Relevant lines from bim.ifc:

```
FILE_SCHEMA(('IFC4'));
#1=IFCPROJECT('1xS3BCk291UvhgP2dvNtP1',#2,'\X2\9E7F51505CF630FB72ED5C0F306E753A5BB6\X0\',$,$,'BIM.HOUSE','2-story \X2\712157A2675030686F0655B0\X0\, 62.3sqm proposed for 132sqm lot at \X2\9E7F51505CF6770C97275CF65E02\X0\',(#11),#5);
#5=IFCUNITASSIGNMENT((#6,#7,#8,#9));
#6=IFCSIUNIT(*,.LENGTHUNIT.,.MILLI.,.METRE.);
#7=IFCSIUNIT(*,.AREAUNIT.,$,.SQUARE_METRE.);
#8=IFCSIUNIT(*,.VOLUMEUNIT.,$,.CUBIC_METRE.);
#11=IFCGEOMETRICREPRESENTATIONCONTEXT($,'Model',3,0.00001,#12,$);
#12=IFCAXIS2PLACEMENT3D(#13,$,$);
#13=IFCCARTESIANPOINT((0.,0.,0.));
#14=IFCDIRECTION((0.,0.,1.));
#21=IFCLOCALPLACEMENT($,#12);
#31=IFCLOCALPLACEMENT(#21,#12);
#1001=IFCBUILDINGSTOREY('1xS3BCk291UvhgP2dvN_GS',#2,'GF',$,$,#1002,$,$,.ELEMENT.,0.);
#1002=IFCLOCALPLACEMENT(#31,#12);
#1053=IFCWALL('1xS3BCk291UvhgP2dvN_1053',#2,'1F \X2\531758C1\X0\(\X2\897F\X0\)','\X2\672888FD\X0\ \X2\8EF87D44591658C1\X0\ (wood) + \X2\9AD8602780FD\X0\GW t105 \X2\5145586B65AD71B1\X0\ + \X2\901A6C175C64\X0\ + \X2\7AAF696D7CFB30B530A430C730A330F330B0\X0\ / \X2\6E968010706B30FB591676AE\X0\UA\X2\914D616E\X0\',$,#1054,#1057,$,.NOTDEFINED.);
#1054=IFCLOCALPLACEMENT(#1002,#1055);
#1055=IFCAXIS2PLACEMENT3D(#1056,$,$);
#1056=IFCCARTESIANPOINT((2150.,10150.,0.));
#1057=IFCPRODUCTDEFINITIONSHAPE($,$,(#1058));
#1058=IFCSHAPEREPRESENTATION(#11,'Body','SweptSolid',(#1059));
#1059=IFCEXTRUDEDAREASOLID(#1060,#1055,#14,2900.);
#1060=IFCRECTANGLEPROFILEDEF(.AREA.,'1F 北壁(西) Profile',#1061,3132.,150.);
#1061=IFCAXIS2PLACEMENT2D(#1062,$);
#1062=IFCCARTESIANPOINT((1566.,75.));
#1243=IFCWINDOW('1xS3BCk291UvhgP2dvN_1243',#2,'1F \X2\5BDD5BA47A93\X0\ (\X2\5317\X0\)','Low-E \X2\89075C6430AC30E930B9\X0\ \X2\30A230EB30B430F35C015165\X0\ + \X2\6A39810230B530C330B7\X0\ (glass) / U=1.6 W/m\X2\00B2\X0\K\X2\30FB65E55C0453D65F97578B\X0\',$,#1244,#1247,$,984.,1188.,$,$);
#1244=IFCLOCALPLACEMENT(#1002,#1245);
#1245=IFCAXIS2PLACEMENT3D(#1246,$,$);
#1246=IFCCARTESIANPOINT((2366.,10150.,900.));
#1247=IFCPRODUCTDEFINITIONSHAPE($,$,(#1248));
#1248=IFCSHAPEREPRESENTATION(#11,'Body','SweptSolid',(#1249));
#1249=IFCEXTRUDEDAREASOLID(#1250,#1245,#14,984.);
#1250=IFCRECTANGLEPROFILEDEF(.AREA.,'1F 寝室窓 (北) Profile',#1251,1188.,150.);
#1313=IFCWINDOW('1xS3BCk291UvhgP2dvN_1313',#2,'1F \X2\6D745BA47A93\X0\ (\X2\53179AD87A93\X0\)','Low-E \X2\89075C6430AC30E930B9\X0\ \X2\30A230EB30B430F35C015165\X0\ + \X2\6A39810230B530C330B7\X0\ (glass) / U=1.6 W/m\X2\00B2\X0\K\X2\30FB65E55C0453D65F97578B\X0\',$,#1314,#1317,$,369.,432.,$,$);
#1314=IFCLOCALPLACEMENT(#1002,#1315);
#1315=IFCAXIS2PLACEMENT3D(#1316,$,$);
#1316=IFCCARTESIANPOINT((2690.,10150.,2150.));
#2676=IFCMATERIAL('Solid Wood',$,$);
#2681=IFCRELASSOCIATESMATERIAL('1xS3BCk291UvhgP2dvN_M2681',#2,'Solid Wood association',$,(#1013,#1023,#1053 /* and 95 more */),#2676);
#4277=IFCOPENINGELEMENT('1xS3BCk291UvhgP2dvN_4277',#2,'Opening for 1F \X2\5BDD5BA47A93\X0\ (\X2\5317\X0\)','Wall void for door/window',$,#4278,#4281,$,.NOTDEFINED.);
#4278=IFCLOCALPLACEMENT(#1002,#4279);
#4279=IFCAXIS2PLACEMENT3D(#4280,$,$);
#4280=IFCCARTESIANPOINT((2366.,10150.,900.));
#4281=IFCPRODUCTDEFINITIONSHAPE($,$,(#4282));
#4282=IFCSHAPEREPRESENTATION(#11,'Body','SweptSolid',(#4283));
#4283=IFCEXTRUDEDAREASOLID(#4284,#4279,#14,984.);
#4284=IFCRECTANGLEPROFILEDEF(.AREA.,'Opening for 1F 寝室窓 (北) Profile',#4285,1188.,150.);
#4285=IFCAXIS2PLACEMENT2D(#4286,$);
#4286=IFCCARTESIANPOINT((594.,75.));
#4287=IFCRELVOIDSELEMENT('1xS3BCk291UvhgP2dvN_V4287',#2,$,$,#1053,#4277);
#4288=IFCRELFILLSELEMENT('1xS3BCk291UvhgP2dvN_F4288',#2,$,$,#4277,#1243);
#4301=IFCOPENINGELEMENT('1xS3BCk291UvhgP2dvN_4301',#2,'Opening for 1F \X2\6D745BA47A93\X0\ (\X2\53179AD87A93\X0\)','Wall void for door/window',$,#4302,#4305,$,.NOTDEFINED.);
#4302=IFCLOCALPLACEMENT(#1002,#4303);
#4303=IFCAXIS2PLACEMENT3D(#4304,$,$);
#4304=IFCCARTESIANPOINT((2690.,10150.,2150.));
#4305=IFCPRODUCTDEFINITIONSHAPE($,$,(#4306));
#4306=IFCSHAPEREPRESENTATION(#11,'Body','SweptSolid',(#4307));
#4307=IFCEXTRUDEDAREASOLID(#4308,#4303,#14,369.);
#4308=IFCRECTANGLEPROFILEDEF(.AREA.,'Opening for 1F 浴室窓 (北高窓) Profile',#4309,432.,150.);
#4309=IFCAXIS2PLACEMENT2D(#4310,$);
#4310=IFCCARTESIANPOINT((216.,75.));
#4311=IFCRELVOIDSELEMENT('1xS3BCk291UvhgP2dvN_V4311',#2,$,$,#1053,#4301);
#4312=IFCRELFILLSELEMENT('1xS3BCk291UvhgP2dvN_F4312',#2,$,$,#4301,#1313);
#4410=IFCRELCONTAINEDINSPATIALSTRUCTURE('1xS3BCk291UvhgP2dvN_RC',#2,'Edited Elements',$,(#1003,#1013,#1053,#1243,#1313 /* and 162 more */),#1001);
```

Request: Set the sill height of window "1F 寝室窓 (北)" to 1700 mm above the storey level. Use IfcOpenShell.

```python
import numpy as np
import ifcopenshell
import ifcopenshell.api.geometry
import ifcopenshell.geom
import ifcopenshell.util.element
import ifcopenshell.util.placement
import ifcopenshell.util.shape
import ifcopenshell.util.unit

model = ifcopenshell.open("bim.ifc")
unit_scale = ifcopenshell.util.unit.calculate_unit_scale(model)

window = model.by_guid("1xS3BCk291UvhgP2dvN_1243")
opening = window.FillsVoids[0].RelatingOpeningElement
storey = ifcopenshell.util.element.get_container(window, ifc_class="IfcBuildingStorey")
level = ifcopenshell.util.placement.get_local_placement(storey.ObjectPlacement)[2, 3]

# The opening's origin need not be at the sill, so measure its lowest point.
shape = ifcopenshell.geom.create_shape(ifcopenshell.geom.settings(), opening)
bottom = ifcopenshell.util.shape.get_shape_bottom_elevation(shape, shape.geometry) / unit_scale
dz = level + 1.7 / unit_scale - bottom

shift = np.array([0.0, 0.0, dz])
# The window is not placed relative to its opening, so move both.
for product in (opening, window):
    matrix = ifcopenshell.util.placement.get_local_placement(product.ObjectPlacement)
    matrix[:3, 3] += shift
    ifcopenshell.api.geometry.edit_object_placement(model, product=product, matrix=matrix, is_si=False)

print(f"moved by {dz * unit_scale:+.3f} m")

model.write("bim_v2.ifc")
```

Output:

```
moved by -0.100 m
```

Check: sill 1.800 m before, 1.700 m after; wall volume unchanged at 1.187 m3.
